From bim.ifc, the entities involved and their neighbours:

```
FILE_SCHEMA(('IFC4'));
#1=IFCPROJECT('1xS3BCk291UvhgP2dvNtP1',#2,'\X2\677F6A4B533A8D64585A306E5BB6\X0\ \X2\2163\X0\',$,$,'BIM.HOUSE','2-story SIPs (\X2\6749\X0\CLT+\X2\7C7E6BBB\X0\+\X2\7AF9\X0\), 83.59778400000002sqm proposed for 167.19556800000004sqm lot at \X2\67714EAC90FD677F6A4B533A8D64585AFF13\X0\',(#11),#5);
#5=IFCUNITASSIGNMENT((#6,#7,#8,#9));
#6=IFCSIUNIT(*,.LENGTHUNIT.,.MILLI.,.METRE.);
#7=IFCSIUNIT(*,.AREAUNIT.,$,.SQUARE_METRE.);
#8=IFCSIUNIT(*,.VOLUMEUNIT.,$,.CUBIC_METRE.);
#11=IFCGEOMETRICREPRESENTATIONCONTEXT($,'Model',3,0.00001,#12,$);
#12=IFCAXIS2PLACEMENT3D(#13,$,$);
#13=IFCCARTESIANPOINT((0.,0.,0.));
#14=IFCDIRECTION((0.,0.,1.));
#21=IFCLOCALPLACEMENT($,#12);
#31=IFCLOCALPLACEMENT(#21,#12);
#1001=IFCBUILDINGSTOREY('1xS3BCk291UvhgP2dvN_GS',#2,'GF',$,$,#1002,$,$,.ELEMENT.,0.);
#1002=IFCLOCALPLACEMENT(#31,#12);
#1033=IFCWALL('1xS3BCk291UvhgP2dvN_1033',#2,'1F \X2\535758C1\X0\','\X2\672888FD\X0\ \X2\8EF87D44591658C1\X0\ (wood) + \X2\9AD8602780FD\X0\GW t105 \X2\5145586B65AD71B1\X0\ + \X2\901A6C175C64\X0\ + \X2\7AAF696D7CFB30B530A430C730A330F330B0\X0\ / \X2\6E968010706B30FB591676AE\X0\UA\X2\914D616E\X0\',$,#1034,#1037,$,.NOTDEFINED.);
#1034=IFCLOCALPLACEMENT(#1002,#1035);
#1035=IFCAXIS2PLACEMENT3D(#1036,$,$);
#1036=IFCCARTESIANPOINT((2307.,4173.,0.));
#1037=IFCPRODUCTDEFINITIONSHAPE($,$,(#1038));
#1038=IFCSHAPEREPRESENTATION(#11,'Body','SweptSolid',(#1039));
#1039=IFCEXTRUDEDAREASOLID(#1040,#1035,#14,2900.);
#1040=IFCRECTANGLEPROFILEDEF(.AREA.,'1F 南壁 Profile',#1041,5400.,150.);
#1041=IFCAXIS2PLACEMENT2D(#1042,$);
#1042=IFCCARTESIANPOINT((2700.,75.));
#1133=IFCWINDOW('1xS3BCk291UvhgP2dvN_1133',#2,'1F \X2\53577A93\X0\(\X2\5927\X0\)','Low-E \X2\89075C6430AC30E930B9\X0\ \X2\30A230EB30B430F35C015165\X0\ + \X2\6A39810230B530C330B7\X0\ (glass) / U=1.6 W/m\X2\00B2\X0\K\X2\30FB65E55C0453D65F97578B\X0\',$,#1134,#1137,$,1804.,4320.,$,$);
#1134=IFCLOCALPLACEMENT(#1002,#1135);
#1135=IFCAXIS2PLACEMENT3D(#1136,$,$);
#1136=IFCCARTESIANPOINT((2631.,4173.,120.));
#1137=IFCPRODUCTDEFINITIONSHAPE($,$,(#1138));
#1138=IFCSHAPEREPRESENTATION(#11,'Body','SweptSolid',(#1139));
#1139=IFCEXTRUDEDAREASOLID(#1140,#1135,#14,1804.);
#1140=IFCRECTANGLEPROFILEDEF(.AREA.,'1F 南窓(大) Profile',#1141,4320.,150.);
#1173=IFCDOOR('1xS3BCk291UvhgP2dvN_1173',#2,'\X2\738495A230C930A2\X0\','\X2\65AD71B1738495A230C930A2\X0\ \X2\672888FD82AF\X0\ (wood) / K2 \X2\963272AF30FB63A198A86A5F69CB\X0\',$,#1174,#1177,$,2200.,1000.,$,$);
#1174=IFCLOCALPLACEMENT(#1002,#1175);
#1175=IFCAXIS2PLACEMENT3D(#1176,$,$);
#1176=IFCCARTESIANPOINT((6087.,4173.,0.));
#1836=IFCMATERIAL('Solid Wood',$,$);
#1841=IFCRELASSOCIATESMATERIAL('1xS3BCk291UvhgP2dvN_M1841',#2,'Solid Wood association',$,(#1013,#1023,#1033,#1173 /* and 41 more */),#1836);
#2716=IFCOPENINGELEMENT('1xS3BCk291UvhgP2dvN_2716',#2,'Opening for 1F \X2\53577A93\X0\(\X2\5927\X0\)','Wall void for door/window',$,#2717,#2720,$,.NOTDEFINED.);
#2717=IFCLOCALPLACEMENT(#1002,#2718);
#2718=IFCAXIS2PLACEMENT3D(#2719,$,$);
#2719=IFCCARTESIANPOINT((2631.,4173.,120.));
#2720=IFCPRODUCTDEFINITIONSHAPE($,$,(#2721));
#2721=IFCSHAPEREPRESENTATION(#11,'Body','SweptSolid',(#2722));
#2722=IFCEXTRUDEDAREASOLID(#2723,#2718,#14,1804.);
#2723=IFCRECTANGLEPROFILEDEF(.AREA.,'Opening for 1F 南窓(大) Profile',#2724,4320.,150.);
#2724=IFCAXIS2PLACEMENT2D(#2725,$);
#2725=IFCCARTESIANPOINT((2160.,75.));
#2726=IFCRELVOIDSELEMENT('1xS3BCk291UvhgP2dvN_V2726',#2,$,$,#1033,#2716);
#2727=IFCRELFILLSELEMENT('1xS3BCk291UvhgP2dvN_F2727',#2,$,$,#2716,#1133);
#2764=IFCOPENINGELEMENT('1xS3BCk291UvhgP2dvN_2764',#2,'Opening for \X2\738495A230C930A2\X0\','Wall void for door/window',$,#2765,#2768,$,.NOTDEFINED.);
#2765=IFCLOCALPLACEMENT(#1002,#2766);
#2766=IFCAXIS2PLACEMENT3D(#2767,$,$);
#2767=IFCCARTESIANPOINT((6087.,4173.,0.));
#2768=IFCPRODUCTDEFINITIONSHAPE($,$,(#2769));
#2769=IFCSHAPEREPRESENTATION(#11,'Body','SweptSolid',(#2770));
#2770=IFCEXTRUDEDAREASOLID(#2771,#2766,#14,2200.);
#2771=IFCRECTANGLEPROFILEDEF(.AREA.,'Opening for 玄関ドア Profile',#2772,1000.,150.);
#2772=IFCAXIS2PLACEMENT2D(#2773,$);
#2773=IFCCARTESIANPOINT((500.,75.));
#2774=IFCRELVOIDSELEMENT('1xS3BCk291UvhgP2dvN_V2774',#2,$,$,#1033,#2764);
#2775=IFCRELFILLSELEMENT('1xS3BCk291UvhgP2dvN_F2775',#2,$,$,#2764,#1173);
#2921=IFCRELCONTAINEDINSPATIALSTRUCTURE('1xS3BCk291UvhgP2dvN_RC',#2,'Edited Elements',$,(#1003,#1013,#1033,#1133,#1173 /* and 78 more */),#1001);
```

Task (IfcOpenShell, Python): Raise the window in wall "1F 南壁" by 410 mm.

```python
import numpy as np
import ifcopenshell
import ifcopenshell.api.geometry
import ifcopenshell.util.placement
import ifcopenshell.util.unit

model = ifcopenshell.open("bim.ifc")
unit_scale = ifcopenshell.util.unit.calculate_unit_scale(model)

window = model.by_guid("1xS3BCk291UvhgP2dvN_1133")
opening = window.FillsVoids[0].RelatingOpeningElement
dz = 410.0

shift = np.array([0.0, 0.0, dz])
# The window is not placed relative to its opening, so move both.
for product in (opening, window):
    matrix = ifcopenshell.util.placement.get_local_placement(product.ObjectPlacement)
    matrix[:3, 3] += shift
    ifcopenshell.api.geometry.edit_object_placement(model, product=product, matrix=matrix, is_si=False)

print(f"moved by {dz * unit_scale:+.3f} m")

model.write("bim-out.ifc")
```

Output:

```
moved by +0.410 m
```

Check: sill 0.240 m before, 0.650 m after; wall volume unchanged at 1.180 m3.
